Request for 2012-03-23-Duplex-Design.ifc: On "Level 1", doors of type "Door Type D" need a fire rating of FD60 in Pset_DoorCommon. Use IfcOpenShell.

First a look at what the model holds.

```python
import ifcopenshell
import ifcopenshell.util.element

model = ifcopenshell.open("2012-03-23-Duplex-Design.ifc")
print(model.schema)
storey = next(s for s in model.by_type("IfcBuildingStorey") if s.Name == "Level 1")
doors = [e for e in ifcopenshell.util.element.get_decomposition(storey) if e.is_a("IfcDoor")]
seen = {}
for e in doors:
    element_type = ifcopenshell.util.element.get_type(e)
    key = (element_type.Name if element_type != e and element_type else None, ifcopenshell.util.element.get_pset(e, "Pset_DoorCommon", "FireRating"))
    seen[key] = seen.get(key, 0) + 1
for (name, value), count in sorted(seen.items(), key=str):
    print(count, "x", name, "|", value)
```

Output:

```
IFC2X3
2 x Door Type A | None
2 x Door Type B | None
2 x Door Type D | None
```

```python
import ifcopenshell
import ifcopenshell.api.pset
import ifcopenshell.util.element

model = ifcopenshell.open("2012-03-23-Duplex-Design.ifc")

storey = next(s for s in model.by_type("IfcBuildingStorey") if s.Name == "Level 1")
doors = [e for e in ifcopenshell.util.element.get_decomposition(storey) if e.is_a("IfcDoor")]

count = 0
for e in doors:
    element_type = ifcopenshell.util.element.get_type(e)
    if element_type in (None, e) or element_type.Name != "Door Type D":
        continue
    # add_pset returns the element's existing set when there is one.
    pset = ifcopenshell.api.pset.add_pset(model, product=e, name="Pset_DoorCommon")
    ifcopenshell.api.pset.edit_pset(model, pset=pset, properties={"FireRating": "FD60"})
    count += 1

print(count, "doors updated")

model.write("2012-03-23-Duplex-Design_v2.ifc")
```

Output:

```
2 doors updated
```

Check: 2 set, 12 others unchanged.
